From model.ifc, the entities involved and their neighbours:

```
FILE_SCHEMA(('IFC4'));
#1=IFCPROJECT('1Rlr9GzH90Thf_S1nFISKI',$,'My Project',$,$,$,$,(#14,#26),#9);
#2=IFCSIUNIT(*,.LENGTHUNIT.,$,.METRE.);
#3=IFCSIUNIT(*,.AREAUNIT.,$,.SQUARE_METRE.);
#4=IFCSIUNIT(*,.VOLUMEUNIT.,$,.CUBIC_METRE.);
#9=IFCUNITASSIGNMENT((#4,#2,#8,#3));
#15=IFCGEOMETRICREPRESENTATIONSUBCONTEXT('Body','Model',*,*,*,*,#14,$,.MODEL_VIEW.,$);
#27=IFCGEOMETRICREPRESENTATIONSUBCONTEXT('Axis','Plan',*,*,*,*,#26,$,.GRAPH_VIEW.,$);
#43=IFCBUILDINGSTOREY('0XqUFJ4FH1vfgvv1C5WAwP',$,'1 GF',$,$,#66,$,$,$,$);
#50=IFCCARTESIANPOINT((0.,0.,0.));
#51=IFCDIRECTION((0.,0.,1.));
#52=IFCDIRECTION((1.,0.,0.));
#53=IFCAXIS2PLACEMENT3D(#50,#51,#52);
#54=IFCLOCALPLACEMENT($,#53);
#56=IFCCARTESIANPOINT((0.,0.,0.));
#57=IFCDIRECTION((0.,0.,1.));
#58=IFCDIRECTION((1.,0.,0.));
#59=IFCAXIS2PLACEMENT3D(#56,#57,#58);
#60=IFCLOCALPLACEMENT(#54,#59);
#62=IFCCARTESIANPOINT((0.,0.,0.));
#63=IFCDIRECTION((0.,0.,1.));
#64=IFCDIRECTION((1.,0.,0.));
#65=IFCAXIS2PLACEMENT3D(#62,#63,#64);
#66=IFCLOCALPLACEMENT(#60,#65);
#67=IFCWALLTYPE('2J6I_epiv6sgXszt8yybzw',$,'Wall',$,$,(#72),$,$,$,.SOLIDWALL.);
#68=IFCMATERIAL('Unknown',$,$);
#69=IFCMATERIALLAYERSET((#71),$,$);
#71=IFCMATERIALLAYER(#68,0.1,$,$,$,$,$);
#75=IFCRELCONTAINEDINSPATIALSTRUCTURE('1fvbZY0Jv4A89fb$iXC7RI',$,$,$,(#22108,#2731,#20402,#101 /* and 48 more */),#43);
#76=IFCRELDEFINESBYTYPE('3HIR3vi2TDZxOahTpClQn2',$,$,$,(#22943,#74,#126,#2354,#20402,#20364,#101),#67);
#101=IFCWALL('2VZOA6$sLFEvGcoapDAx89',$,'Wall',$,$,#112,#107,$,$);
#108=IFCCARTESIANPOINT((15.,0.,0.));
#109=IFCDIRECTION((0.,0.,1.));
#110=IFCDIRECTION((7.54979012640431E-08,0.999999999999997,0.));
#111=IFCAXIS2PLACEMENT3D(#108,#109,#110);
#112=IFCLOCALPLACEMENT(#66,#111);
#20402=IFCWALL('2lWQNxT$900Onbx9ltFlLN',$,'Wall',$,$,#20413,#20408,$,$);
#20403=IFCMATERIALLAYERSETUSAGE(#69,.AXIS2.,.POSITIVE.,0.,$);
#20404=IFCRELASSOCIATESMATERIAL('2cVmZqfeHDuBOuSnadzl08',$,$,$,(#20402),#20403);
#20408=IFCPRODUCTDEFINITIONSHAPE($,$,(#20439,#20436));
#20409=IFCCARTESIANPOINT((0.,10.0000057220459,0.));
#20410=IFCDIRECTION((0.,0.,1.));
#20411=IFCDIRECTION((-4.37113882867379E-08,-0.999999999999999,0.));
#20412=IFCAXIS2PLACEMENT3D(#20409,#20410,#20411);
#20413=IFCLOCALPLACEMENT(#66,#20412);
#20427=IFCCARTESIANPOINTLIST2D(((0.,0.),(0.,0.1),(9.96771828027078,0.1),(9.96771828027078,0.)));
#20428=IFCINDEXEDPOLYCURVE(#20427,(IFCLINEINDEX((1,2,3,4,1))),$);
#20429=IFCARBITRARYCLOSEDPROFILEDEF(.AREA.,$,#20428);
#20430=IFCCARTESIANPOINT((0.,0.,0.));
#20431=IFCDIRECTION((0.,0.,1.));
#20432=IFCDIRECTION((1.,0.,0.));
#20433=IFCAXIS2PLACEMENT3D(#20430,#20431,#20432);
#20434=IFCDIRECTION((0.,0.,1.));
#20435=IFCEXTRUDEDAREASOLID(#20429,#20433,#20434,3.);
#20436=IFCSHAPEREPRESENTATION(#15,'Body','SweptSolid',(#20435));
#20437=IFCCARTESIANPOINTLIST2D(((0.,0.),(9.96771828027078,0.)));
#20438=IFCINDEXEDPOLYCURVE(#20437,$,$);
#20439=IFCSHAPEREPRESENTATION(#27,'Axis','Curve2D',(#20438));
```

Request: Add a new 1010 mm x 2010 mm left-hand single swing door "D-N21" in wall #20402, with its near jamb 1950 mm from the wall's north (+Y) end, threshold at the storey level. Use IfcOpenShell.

```python
import numpy as np
import ifcopenshell
import ifcopenshell.api.feature
import ifcopenshell.api.geometry
import ifcopenshell.api.root
import ifcopenshell.api.spatial
import ifcopenshell.geom
import ifcopenshell.util.element
import ifcopenshell.util.placement
import ifcopenshell.util.representation
import ifcopenshell.util.shape
import ifcopenshell.util.unit

model = ifcopenshell.open("model.ifc")
unit_scale = ifcopenshell.util.unit.calculate_unit_scale(model)
settings = ifcopenshell.geom.settings()


def volume(element):
    """Net volume in cubic metres, openings subtracted."""
    shape = ifcopenshell.geom.create_shape(settings, element)
    return ifcopenshell.util.shape.get_volume(shape.geometry)


wall = model.by_guid("2lWQNxT$900Onbx9ltFlLN")
storey = ifcopenshell.util.element.get_container(wall, ifc_class="IfcBuildingStorey")
context = ifcopenshell.util.representation.get_context(model, "Model", "Body", "MODEL_VIEW")
before = volume(wall)

width, height, from_end, sill = 1.01, 2.01, 1.95, 0.0  # metres

# The wall runs along its own X axis, and the end named is its -X end.
wall_shape = ifcopenshell.geom.create_shape(settings, wall)
x, y, z = ifcopenshell.util.shape.get_vertices(wall_shape.geometry).T
start = x.min() + from_end
face, thickness = float(y.min()), float(y.max() - y.min())
wall_matrix = ifcopenshell.util.placement.get_local_placement(wall.ObjectPlacement)
level = ifcopenshell.util.placement.get_local_placement(storey.ObjectPlacement)[2, 3]


def in_wall(x, y):
    """Placement at x, y metres in the wall's axes, at sill height."""
    matrix = wall_matrix.copy()
    matrix[:, 3] = wall_matrix @ np.array([x / unit_scale, y / unit_scale, 0.0, 1.0])
    matrix[2, 3] = level + sill / unit_scale
    return matrix


# Opening: a box that overshoots both wall faces by 50 mm.
opening = ifcopenshell.api.root.create_entity(model, ifc_class="IfcOpeningElement", predefined_type="OPENING")
box = ifcopenshell.api.geometry.add_wall_representation(
    model, context=context, length=width, height=height, thickness=thickness + 0.1
)
ifcopenshell.api.geometry.assign_representation(model, product=opening, representation=box)
ifcopenshell.api.geometry.edit_object_placement(model, product=opening, matrix=in_wall(start, face - 0.05), is_si=False)
ifcopenshell.api.feature.add_feature(model, feature=opening, element=wall)

door = ifcopenshell.api.root.create_entity(model, ifc_class="IfcDoor", name="D-N21", predefined_type="DOOR")
door.OverallWidth, door.OverallHeight = width / unit_scale, height / unit_scale
door.OperationType = "SINGLE_SWING_LEFT"
body = ifcopenshell.api.geometry.add_door_representation(
    model,
    context=context,
    overall_width=door.OverallWidth,
    overall_height=door.OverallHeight,
    operation_type="SINGLE_SWING_LEFT",
    lining_properties={"LiningDepth": thickness / unit_scale, "ThresholdDepth": thickness / unit_scale},
)
ifcopenshell.api.geometry.assign_representation(model, product=door, representation=body)
ifcopenshell.api.spatial.assign_container(model, products=[door], relating_structure=storey)
ifcopenshell.api.feature.add_filling(model, opening=opening, element=door)

# The lining spans the wall, so the door starts at the wall face.
ifcopenshell.api.geometry.edit_object_placement(model, product=door, matrix=in_wall(start, face), is_si=False)

after = volume(wall)

print(f"wall volume {before:.3f} -> {after:.3f} m3")

model.write("model-out.ifc")
```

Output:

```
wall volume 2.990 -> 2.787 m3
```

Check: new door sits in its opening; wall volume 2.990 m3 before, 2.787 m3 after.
